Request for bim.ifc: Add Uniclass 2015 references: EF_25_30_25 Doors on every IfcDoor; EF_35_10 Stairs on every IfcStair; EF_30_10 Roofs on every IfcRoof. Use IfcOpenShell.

First a look at what the model holds.

```python
import ifcopenshell

model = ifcopenshell.open("bim.ifc")
print(model.schema)
print("classifications:", [c.Name for c in model.by_type("IfcClassification")])
for ifc_class in ("IfcDoor", "IfcRoof", "IfcStair", "IfcWall", "IfcWindow"):
    print(ifc_class, len(model.by_type(ifc_class)))
```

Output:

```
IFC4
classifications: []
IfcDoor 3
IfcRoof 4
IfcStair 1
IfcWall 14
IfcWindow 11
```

```python
import ifcopenshell
import ifcopenshell.api.classification

model = ifcopenshell.open("bim.ifc")

system = ifcopenshell.api.classification.add_classification(model, classification="Uniclass 2015")

codes = {
    "IfcDoor": ("EF_25_30_25", "Doors"),
    "IfcStair": ("EF_35_10", "Stairs"),
    "IfcRoof": ("EF_30_10", "Roofs"),
}
for ifc_class, (code, name) in codes.items():
    products = model.by_type(ifc_class)
    ifcopenshell.api.classification.add_reference(
        model, products=products, classification=system, identification=code, name=name
    )
    print(code, len(products))

model.write("bim_edited.ifc")
```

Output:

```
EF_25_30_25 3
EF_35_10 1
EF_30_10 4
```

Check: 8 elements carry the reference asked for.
